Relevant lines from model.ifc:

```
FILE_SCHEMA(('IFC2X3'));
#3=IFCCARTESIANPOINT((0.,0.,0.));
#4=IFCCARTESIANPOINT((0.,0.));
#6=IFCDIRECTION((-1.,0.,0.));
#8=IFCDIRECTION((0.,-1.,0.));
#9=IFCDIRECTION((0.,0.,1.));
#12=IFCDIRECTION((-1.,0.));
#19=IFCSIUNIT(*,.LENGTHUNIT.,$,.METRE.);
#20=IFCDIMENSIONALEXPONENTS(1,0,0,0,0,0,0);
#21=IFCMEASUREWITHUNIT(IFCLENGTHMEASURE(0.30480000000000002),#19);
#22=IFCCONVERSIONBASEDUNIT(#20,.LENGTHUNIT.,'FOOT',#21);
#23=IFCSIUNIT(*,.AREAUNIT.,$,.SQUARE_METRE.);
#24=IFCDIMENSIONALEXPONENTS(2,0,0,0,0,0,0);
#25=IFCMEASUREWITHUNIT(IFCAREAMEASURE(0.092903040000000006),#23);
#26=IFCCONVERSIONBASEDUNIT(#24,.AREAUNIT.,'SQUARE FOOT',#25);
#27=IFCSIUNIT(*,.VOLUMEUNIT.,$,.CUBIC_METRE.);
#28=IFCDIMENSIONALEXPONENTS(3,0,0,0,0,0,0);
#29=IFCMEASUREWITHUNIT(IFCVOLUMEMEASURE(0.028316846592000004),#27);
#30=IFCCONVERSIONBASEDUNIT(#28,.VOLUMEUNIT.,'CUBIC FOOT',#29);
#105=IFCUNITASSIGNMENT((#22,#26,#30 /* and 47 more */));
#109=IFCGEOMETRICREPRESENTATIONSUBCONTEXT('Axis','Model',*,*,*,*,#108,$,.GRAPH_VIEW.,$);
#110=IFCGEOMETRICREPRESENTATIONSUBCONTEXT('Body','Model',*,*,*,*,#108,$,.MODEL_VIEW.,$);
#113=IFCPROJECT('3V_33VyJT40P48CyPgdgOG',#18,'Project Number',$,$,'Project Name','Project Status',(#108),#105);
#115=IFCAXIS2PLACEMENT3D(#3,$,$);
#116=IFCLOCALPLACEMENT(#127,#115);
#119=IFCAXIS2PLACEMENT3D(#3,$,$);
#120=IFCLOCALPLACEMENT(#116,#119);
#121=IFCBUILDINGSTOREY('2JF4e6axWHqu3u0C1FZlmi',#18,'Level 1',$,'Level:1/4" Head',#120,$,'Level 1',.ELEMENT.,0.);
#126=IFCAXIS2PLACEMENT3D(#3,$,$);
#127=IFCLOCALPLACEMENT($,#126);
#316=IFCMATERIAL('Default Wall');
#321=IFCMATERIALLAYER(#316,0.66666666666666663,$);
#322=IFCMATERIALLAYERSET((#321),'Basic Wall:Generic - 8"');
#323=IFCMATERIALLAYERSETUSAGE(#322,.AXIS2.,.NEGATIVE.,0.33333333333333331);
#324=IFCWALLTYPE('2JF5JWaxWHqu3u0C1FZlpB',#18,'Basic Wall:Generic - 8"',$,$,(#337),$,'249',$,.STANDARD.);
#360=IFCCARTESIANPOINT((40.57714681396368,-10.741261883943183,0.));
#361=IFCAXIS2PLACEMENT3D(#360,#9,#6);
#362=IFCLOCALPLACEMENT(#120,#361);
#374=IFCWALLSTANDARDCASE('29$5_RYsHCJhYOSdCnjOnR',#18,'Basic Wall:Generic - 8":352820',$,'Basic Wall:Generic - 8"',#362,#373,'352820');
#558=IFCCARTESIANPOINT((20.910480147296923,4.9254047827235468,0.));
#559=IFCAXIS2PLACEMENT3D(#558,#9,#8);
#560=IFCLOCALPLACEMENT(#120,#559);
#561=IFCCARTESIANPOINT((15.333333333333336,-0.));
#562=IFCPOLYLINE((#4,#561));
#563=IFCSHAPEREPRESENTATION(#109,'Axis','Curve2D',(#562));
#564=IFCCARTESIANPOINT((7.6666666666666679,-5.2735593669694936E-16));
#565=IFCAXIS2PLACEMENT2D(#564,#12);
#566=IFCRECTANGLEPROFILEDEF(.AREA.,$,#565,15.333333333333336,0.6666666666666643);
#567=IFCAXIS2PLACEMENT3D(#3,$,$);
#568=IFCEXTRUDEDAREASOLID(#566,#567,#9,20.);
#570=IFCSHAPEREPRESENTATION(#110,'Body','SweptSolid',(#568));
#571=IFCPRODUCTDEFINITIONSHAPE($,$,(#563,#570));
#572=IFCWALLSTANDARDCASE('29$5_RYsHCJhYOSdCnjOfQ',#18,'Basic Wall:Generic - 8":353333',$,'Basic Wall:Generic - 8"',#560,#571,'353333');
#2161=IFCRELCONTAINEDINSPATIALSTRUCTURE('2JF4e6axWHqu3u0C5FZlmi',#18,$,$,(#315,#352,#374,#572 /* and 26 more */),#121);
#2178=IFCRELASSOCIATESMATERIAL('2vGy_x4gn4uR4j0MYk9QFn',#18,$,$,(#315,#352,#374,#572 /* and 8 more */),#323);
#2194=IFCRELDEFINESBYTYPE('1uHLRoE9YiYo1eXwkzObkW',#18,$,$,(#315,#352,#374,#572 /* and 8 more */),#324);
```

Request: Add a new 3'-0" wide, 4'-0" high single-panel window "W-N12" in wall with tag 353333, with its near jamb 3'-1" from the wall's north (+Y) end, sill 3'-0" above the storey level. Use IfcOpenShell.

```python
import numpy as np
import ifcopenshell
import ifcopenshell.api.feature
import ifcopenshell.api.geometry
import ifcopenshell.api.root
import ifcopenshell.api.spatial
import ifcopenshell.api.type
import ifcopenshell.geom
import ifcopenshell.util.element
import ifcopenshell.util.placement
import ifcopenshell.util.representation
import ifcopenshell.util.shape
import ifcopenshell.util.unit

model = ifcopenshell.open("model.ifc")
unit_scale = ifcopenshell.util.unit.calculate_unit_scale(model)
settings = ifcopenshell.geom.settings()


def volume(element):
    """Net volume in cubic metres, openings subtracted."""
    shape = ifcopenshell.geom.create_shape(settings, element)
    return ifcopenshell.util.shape.get_volume(shape.geometry)


wall = model.by_guid("29$5_RYsHCJhYOSdCnjOfQ")
storey = ifcopenshell.util.element.get_container(wall, ifc_class="IfcBuildingStorey")
context = ifcopenshell.util.representation.get_context(model, "Model", "Body", "MODEL_VIEW")
before = volume(wall)

width, height, from_end, sill = 0.9144, 1.2192, 0.9398, 0.9144  # metres

# The wall runs along its own X axis, and the end named is its -X end.
wall_shape = ifcopenshell.geom.create_shape(settings, wall)
x, y, z = ifcopenshell.util.shape.get_vertices(wall_shape.geometry).T
start = x.min() + from_end
face, thickness = float(y.min()), float(y.max() - y.min())
wall_matrix = ifcopenshell.util.placement.get_local_placement(wall.ObjectPlacement)
level = ifcopenshell.util.placement.get_local_placement(storey.ObjectPlacement)[2, 3]


def in_wall(x, y):
    """Placement at x, y metres in the wall's axes, at sill height."""
    matrix = wall_matrix.copy()
    matrix[:, 3] = wall_matrix @ np.array([x / unit_scale, y / unit_scale, 0.0, 1.0])
    matrix[2, 3] = level + sill / unit_scale
    return matrix


# Opening: a box that overshoots both wall faces by 50 mm.
opening = ifcopenshell.api.root.create_entity(model, ifc_class="IfcOpeningElement")
box = ifcopenshell.api.geometry.add_wall_representation(
    model, context=context, length=width, height=height, thickness=thickness + 0.1
)
ifcopenshell.api.geometry.assign_representation(model, product=opening, representation=box)
ifcopenshell.api.geometry.edit_object_placement(model, product=opening, matrix=in_wall(start, face - 0.05), is_si=False)
ifcopenshell.api.feature.add_feature(model, feature=opening, element=wall)

window = ifcopenshell.api.root.create_entity(model, ifc_class="IfcWindow", name="W-N12")
window.OverallWidth, window.OverallHeight = width / unit_scale, height / unit_scale
body = ifcopenshell.api.geometry.add_window_representation(
    model,
    context=context,
    overall_width=window.OverallWidth,
    overall_height=window.OverallHeight,
    partition_type="SINGLE_PANEL",
)
ifcopenshell.api.geometry.assign_representation(model, product=window, representation=body)
ifcopenshell.api.spatial.assign_container(model, products=[window], relating_structure=storey)
fills = ifcopenshell.api.feature.add_filling(model, opening=opening, element=window)
fills.OwnerHistory = window.OwnerHistory  # required in IFC2X3

# IFC2X3 keeps the operation on the window style.
style = ifcopenshell.api.root.create_entity(model, ifc_class="IfcWindowStyle", name="W-N12")
style.OperationType, style.ConstructionType = "SINGLE_PANEL", "NOTDEFINED"
style.ParameterTakesPrecedence = style.Sizeable = False
ifcopenshell.api.type.assign_type(model, related_objects=[window], relating_type=style)

# Centre the window in the wall's thickness.
ifcopenshell.api.geometry.edit_object_placement(model, product=window, matrix=in_wall(start, face), is_si=False)
window_shape = ifcopenshell.geom.create_shape(settings, window)
depth = ifcopenshell.util.shape.get_vertices(window_shape.geometry)[:, 1]
offset = face + thickness / 2 - (depth.min() + depth.max()) / 2
ifcopenshell.api.geometry.edit_object_placement(model, product=window, matrix=in_wall(start, offset), is_si=False)

after = volume(wall)

print(f"wall volume {before:.3f} -> {after:.3f} m3")

model.write("model_updated.ifc")
```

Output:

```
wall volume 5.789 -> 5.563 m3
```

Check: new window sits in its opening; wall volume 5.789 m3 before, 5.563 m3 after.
